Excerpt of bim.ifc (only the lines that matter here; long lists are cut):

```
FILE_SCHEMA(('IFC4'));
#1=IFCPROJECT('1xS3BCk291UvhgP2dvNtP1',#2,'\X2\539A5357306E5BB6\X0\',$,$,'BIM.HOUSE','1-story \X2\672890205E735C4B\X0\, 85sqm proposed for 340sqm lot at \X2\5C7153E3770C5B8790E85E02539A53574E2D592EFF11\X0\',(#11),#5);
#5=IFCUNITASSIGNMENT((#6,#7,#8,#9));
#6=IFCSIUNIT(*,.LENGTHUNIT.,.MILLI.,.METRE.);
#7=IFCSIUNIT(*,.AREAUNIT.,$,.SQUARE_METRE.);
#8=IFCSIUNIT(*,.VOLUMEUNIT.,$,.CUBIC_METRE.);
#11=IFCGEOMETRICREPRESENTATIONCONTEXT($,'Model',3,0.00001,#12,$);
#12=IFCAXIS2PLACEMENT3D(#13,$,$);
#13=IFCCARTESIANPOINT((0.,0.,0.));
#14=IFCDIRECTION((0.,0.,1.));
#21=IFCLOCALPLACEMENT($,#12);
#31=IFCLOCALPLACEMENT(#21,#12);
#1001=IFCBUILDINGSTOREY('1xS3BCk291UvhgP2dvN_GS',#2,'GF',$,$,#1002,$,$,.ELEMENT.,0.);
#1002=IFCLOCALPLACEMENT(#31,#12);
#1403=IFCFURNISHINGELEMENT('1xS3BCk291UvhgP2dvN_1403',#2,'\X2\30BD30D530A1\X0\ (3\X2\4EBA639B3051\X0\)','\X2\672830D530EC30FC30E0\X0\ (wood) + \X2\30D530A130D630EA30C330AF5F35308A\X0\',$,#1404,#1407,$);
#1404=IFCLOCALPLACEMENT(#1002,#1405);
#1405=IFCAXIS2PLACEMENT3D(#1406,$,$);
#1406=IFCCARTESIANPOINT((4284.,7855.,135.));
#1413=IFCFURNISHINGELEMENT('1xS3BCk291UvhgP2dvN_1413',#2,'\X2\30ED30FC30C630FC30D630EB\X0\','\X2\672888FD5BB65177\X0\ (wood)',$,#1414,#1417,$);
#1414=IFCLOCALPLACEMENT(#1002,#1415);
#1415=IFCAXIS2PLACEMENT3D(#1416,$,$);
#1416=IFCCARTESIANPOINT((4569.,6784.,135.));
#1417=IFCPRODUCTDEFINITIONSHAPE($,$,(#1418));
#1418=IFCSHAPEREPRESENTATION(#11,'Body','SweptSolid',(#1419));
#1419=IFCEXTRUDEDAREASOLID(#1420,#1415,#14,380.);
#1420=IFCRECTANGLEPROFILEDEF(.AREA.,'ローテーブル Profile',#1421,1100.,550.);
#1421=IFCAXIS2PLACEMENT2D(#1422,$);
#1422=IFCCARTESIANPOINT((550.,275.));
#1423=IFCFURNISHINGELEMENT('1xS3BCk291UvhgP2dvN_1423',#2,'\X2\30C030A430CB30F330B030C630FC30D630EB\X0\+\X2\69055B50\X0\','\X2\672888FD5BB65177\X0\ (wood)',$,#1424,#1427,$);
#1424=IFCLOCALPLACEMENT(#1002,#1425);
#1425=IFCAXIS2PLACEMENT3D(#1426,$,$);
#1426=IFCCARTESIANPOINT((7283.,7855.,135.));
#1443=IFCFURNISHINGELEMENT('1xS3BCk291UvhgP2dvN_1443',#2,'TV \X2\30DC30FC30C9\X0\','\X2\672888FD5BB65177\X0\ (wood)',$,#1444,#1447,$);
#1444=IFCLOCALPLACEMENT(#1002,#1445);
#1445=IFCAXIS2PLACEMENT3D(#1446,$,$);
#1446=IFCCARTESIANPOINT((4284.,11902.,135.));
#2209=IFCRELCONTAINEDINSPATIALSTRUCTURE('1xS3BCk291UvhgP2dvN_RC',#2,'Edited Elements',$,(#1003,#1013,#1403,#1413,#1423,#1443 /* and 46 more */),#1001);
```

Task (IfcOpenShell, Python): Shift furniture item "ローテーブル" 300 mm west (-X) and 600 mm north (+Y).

```python
import ifcopenshell
import ifcopenshell.api.geometry
import ifcopenshell.util.placement
import ifcopenshell.util.unit

model = ifcopenshell.open("bim.ifc")
unit_scale = ifcopenshell.util.unit.calculate_unit_scale(model)

item = model.by_guid("1xS3BCk291UvhgP2dvN_1413")
matrix = ifcopenshell.util.placement.get_local_placement(item.ObjectPlacement)
matrix[0, 3] -= 0.3 / unit_scale
matrix[1, 3] += 0.6 / unit_scale
ifcopenshell.api.geometry.edit_object_placement(model, product=item, matrix=matrix, is_si=False)

print(ifcopenshell.util.placement.get_local_placement(item.ObjectPlacement).round(3) + 0.0)

model.write("bim-out.ifc")
```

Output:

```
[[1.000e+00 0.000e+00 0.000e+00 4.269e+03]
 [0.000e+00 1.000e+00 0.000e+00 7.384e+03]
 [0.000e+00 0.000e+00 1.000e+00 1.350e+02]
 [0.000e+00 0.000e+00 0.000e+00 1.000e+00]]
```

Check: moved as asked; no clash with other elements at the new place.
